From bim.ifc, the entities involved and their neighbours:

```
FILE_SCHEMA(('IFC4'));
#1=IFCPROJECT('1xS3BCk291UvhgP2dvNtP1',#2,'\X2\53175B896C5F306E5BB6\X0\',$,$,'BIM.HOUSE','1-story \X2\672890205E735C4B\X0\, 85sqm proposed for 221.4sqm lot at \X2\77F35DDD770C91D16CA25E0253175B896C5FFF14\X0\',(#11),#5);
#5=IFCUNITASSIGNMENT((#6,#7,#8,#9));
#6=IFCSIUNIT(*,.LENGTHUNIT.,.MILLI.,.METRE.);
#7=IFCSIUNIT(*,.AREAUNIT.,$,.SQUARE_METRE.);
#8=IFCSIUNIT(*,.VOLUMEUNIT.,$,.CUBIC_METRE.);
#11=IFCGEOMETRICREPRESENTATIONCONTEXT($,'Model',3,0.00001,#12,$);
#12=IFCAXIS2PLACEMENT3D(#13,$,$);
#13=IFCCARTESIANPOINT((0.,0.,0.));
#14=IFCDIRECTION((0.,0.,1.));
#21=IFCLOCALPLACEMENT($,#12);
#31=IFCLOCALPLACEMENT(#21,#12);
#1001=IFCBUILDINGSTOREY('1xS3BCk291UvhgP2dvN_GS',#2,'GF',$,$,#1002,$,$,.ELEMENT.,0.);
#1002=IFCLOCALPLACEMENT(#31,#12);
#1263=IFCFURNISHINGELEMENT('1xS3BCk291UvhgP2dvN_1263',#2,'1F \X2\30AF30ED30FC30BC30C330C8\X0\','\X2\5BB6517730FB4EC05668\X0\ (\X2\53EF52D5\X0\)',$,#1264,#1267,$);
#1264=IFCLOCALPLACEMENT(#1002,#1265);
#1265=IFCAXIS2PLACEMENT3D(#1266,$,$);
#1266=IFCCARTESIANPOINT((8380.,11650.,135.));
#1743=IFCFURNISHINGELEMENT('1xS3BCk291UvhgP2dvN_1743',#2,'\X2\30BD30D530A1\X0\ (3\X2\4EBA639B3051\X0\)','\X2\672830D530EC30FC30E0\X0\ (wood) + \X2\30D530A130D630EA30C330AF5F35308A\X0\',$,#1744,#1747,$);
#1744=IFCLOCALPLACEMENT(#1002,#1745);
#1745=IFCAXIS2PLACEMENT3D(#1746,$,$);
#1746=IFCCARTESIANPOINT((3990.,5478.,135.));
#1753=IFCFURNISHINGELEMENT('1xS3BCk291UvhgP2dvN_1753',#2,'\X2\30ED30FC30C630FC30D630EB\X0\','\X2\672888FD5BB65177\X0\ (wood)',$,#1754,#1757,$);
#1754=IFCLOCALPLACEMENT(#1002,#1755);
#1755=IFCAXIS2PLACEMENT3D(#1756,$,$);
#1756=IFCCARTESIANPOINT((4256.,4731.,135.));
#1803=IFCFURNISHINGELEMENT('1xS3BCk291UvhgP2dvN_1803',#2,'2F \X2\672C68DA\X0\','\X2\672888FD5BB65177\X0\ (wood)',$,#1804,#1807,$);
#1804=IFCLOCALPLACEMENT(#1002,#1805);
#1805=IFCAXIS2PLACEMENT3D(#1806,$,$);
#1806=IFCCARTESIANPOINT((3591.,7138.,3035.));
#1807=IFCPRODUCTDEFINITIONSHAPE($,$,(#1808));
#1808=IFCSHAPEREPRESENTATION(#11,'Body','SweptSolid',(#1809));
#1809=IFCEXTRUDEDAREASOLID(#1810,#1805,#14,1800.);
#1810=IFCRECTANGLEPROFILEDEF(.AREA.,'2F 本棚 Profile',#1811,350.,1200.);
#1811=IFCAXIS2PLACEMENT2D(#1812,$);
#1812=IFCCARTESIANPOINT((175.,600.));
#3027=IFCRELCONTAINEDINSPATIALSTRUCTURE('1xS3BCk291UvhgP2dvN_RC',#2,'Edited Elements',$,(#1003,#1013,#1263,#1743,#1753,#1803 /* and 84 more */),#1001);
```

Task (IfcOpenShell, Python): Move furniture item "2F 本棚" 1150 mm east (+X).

```python
import ifcopenshell
import ifcopenshell.api.geometry
import ifcopenshell.util.placement
import ifcopenshell.util.unit

model = ifcopenshell.open("bim.ifc")
unit_scale = ifcopenshell.util.unit.calculate_unit_scale(model)

item = model.by_guid("1xS3BCk291UvhgP2dvN_1803")
matrix = ifcopenshell.util.placement.get_local_placement(item.ObjectPlacement)
matrix[0, 3] += 1.15 / unit_scale
ifcopenshell.api.geometry.edit_object_placement(model, product=item, matrix=matrix, is_si=False)

print(ifcopenshell.util.placement.get_local_placement(item.ObjectPlacement).round(3) + 0.0)

model.write("bim-out.ifc")
```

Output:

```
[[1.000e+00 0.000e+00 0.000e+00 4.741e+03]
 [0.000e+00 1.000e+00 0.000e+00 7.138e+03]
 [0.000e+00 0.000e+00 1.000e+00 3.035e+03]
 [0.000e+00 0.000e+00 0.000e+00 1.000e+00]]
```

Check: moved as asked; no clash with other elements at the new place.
